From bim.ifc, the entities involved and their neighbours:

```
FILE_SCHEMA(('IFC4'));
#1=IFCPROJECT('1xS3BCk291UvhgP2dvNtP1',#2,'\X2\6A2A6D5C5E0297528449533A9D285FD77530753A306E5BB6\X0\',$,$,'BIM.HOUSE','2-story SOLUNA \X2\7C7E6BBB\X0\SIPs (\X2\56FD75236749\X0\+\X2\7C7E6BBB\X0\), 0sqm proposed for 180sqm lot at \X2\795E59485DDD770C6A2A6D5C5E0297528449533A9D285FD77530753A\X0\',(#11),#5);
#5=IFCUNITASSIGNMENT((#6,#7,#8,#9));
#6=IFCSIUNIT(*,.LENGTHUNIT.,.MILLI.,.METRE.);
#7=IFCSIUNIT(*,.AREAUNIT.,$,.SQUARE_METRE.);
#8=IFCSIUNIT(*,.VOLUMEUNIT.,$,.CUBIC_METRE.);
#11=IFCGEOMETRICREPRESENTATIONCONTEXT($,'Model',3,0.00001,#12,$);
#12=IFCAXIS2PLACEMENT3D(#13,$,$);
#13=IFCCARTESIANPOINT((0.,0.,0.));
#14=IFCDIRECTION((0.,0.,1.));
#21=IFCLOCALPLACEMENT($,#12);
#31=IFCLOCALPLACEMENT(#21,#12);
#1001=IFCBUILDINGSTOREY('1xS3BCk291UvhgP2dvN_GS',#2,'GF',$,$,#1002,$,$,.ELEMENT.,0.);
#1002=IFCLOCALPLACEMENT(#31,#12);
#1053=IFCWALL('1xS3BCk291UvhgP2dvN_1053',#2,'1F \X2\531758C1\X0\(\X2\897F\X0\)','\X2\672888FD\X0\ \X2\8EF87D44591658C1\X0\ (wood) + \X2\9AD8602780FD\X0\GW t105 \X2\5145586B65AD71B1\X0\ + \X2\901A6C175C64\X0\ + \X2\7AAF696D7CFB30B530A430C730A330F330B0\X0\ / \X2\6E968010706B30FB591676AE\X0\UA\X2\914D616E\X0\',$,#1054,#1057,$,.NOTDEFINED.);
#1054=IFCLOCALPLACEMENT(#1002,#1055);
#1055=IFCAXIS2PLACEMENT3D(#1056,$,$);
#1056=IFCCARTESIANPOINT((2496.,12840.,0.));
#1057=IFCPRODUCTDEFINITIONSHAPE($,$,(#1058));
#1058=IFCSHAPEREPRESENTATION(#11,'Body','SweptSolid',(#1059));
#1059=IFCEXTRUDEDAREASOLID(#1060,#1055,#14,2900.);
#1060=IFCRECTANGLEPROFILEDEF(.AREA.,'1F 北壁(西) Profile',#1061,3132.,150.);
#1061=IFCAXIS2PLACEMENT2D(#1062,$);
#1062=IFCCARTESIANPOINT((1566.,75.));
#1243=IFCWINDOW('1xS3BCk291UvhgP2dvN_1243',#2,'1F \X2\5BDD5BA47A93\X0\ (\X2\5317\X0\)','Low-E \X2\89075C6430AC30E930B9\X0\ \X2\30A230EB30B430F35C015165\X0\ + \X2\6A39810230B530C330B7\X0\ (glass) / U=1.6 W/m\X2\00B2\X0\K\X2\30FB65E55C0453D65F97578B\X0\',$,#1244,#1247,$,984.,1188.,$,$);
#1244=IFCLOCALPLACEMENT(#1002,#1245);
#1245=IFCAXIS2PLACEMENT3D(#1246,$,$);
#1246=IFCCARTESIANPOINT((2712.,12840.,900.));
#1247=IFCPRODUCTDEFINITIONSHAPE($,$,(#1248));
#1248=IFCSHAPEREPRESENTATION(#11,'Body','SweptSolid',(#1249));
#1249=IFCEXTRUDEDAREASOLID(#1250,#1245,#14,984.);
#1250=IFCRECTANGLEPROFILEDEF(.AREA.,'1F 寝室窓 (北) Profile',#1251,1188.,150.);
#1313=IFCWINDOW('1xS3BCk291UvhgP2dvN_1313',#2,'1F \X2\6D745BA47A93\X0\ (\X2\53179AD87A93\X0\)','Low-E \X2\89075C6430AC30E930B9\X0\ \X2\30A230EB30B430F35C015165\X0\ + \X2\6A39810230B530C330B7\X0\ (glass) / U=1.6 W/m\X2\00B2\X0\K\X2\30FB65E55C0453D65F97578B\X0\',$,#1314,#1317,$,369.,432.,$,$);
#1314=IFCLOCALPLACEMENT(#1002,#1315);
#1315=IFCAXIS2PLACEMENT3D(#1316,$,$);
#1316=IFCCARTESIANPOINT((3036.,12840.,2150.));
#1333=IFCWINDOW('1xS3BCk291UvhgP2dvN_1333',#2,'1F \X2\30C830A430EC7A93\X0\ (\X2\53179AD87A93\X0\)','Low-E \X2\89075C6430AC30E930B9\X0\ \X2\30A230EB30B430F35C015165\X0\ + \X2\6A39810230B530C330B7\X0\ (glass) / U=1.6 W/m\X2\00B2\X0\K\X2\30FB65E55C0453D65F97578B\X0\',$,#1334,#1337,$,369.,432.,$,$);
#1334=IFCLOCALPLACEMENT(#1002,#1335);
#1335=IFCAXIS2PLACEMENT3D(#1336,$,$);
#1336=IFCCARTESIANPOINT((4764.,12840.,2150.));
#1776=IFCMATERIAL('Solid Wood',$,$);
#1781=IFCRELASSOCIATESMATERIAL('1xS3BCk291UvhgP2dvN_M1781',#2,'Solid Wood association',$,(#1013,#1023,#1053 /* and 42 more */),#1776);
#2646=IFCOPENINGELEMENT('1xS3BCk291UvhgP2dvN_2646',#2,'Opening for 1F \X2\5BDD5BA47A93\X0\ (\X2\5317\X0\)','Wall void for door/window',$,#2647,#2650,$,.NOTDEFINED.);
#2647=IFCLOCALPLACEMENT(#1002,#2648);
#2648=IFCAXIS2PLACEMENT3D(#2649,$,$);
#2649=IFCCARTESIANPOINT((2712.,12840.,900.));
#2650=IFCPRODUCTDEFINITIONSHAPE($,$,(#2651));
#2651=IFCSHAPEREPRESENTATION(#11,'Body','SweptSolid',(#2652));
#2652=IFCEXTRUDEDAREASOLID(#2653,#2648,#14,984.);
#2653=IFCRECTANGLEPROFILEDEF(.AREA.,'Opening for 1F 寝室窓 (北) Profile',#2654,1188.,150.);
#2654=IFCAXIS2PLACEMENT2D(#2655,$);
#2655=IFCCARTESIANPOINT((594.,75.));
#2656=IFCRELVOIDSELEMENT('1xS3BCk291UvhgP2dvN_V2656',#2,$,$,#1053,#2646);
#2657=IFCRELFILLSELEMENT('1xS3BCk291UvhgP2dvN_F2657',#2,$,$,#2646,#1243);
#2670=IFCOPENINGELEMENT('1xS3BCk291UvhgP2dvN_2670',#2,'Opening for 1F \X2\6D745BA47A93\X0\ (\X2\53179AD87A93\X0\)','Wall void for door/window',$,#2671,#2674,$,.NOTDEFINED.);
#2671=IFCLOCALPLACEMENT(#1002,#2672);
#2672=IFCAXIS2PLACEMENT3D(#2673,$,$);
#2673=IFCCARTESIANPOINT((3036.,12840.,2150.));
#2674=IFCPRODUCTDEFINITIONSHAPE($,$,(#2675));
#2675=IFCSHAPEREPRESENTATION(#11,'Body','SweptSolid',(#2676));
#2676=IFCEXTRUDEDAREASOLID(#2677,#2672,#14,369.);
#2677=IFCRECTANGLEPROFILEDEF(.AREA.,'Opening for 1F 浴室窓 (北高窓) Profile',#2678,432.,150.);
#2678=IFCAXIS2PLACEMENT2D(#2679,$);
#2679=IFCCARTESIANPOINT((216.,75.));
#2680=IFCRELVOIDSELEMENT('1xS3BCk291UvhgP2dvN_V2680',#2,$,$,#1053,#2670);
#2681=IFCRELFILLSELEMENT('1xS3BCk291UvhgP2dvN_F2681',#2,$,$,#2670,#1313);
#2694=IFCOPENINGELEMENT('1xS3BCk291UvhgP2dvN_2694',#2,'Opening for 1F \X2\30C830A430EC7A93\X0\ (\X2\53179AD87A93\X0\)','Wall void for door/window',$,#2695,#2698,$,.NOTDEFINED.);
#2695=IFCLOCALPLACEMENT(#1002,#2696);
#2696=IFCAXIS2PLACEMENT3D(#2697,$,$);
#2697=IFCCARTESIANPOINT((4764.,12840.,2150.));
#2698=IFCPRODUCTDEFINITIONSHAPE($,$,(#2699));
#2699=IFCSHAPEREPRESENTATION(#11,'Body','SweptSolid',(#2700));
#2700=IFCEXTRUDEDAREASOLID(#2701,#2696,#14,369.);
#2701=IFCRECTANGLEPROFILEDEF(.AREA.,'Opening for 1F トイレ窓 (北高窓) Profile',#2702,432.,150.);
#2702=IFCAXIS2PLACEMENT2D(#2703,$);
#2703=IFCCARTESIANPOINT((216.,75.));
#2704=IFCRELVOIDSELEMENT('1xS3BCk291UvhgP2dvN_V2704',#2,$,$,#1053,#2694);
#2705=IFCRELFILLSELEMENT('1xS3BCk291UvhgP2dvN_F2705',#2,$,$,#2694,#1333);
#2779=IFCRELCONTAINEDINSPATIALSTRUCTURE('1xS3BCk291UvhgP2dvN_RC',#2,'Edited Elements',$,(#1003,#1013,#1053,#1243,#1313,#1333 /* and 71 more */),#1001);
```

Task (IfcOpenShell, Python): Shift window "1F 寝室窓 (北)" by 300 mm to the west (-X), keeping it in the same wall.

```python
import ifcopenshell
import ifcopenshell.api.geometry
import ifcopenshell.util.placement
import ifcopenshell.util.unit

model = ifcopenshell.open("bim.ifc")
unit_scale = ifcopenshell.util.unit.calculate_unit_scale(model)

window = model.by_id(1243)
opening = window.FillsVoids[0].RelatingOpeningElement
wall = opening.VoidsElements[0].RelatingBuildingElement

wall_matrix = ifcopenshell.util.placement.get_local_placement(wall.ObjectPlacement)
shift = wall_matrix[:3, 0] * -0.3 / unit_scale
before = ifcopenshell.util.placement.get_local_placement(window.ObjectPlacement)[:3, 3].copy()

# The window is not placed relative to its opening, so move both.
for product in (opening, window):
    matrix = ifcopenshell.util.placement.get_local_placement(product.ObjectPlacement)
    matrix[:3, 3] += shift
    ifcopenshell.api.geometry.edit_object_placement(model, product=product, matrix=matrix, is_si=False)

after = ifcopenshell.util.placement.get_local_placement(window.ObjectPlacement)[:3, 3]
print("window moved by", (after - before).round(3) + 0.0)

model.write("bim_updated.ifc")
```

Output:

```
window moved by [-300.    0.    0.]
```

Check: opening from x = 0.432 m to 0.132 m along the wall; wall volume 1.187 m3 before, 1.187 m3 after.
